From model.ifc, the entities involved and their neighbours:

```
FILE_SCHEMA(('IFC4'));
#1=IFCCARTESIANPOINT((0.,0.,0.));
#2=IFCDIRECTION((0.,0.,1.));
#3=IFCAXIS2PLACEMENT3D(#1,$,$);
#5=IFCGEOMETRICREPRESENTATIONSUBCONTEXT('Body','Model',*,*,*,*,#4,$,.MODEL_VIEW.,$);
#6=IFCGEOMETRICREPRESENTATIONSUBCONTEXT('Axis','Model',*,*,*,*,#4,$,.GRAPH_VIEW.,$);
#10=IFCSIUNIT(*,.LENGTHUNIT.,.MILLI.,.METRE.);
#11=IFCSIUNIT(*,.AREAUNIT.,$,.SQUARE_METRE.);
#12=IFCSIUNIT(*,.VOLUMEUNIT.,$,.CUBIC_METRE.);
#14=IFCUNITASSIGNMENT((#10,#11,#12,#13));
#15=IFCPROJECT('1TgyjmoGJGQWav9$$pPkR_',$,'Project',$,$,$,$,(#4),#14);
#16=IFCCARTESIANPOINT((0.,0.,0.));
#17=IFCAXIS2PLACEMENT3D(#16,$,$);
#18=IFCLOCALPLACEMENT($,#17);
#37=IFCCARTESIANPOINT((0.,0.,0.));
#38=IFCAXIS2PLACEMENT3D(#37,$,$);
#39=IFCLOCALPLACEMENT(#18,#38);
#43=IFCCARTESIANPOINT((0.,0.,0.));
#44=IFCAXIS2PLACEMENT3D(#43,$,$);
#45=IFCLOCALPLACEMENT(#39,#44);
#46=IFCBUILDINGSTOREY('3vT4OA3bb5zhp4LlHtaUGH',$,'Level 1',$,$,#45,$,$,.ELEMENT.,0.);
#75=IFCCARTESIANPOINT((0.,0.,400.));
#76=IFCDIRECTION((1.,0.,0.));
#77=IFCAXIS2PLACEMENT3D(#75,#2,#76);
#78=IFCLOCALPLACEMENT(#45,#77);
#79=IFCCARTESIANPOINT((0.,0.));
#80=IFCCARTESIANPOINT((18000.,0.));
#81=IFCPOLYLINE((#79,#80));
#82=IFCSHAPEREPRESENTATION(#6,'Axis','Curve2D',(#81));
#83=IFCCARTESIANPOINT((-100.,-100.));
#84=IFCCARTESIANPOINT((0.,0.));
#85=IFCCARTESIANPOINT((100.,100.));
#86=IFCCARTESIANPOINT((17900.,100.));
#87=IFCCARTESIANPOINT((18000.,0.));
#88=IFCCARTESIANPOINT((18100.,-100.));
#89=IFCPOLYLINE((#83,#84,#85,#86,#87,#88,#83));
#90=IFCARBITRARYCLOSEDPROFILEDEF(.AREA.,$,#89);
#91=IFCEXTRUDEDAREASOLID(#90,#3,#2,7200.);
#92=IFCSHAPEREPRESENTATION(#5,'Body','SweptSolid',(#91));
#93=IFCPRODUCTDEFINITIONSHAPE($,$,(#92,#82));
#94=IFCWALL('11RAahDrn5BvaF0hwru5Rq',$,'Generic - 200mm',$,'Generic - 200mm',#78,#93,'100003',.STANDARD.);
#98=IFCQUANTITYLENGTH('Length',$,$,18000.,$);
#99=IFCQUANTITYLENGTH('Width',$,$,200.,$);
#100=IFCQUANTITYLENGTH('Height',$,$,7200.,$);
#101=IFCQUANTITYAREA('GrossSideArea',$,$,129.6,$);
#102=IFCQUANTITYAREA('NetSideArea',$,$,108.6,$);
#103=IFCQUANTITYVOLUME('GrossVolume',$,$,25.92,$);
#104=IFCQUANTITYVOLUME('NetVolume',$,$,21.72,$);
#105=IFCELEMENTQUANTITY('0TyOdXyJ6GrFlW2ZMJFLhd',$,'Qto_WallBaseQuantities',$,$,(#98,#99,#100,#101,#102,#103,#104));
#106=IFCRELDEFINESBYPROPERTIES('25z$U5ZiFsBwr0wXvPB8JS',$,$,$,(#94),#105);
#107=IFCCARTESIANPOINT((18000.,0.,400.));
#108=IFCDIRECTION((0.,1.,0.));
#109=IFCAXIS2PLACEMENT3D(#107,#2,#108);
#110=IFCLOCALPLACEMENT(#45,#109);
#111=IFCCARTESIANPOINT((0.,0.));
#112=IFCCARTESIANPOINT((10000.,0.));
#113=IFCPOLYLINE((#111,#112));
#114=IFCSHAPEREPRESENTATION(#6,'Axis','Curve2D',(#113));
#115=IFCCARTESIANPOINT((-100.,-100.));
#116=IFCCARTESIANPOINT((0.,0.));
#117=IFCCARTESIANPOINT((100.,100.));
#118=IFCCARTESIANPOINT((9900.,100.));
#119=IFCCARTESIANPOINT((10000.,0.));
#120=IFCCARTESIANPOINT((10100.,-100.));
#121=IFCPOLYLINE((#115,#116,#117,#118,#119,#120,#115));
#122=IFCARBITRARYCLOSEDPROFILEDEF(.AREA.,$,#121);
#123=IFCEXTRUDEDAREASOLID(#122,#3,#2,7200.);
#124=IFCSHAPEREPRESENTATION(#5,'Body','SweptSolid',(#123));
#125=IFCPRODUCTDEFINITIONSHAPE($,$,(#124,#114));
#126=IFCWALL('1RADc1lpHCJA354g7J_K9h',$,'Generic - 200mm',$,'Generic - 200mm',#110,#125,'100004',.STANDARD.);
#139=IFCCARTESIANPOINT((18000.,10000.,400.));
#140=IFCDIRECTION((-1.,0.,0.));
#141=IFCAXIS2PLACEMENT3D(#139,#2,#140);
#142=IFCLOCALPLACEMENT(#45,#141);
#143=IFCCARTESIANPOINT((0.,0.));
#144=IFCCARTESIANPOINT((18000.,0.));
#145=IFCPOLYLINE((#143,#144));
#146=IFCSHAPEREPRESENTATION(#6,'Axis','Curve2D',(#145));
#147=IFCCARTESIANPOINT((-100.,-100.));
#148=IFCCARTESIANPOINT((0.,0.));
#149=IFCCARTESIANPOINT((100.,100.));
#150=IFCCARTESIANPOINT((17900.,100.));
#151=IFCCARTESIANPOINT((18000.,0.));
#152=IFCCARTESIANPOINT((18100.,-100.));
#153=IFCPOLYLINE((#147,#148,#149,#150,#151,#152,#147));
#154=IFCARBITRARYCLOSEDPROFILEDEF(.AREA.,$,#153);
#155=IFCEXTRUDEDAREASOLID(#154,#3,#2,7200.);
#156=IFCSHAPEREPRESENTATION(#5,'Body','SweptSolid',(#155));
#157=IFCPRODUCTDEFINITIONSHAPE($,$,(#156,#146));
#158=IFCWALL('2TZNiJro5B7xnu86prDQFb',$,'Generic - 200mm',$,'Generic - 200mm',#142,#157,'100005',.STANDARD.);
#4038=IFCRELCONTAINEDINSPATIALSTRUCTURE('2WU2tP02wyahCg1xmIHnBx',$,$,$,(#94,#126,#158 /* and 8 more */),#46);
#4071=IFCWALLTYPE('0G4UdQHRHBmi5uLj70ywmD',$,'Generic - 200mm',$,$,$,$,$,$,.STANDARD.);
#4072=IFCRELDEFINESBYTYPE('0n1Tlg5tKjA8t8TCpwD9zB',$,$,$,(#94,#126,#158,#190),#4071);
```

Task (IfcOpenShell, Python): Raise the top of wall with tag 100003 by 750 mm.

```python
import ifcopenshell
import ifcopenshell.api.pset
import ifcopenshell.geom
import ifcopenshell.util.element
import ifcopenshell.util.representation
import ifcopenshell.util.shape
import ifcopenshell.util.unit

model = ifcopenshell.open("model.ifc")
unit_scale = ifcopenshell.util.unit.calculate_unit_scale(model)
area_scale = ifcopenshell.util.unit.calculate_unit_scale(model, "AREAUNIT")
volume_scale = ifcopenshell.util.unit.calculate_unit_scale(model, "VOLUMEUNIT")
settings = ifcopenshell.geom.settings()


def volume(element):
    """Net volume in cubic metres, openings subtracted."""
    shape = ifcopenshell.geom.create_shape(settings, element)
    return ifcopenshell.util.shape.get_volume(shape.geometry)


wall = model.by_guid("11RAahDrn5BvaF0hwru5Rq")
before = volume(wall)

body = ifcopenshell.util.representation.get_representation(wall, "Model", "Body")
solid = body.Items[0]
old_height = solid.Depth
solid.Depth += 0.75 / unit_scale
after = volume(wall)
thickness = 0.2  # wall thickness in metres

# Update the stored height, areas and volumes.
qto = model.by_id(ifcopenshell.util.element.get_pset(wall, "Qto_WallBaseQuantities", should_inherit=False)["id"])
ifcopenshell.api.pset.edit_qto(model, qto=qto, properties={
    "Height": solid.Depth,
    "GrossSideArea": ifcopenshell.util.element.get_pset(wall, "Qto_WallBaseQuantities", "GrossSideArea") * solid.Depth / old_height,
    "NetSideArea": after / thickness / area_scale,
    "GrossVolume": ifcopenshell.util.element.get_pset(wall, "Qto_WallBaseQuantities", "GrossVolume") * solid.Depth / old_height,
    "NetVolume": after / volume_scale,
})

print(f"height {old_height:g} -> {solid.Depth:g}, volume {before:.3f} -> {after:.3f} m3")

model.write("model_edited.ifc")
```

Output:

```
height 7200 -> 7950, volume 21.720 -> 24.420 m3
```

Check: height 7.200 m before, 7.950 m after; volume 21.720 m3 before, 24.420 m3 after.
